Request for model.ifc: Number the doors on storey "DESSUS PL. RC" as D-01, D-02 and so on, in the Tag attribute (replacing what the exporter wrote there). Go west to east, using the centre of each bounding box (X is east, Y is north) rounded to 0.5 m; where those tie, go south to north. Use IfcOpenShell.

First a look at what the model holds.

```python
import ifcopenshell
import ifcopenshell.util.element
import ifcopenshell.util.placement

model = ifcopenshell.open("model.ifc")
print(model.schema)
storey = next(s for s in model.by_type("IfcBuildingStorey") if s.Name == "DESSUS PL. RC")
doors = [e for e in ifcopenshell.util.element.get_decomposition(storey) if e.is_a("IfcDoor")]
for e in sorted(doors, key=lambda e: e.id()):
    origin = ifcopenshell.util.placement.get_local_placement(e.ObjectPlacement)[:3, 3]
    print(e.id(), e.Tag, e.Name, origin.round(2) + 0.0, sep=" | ")
```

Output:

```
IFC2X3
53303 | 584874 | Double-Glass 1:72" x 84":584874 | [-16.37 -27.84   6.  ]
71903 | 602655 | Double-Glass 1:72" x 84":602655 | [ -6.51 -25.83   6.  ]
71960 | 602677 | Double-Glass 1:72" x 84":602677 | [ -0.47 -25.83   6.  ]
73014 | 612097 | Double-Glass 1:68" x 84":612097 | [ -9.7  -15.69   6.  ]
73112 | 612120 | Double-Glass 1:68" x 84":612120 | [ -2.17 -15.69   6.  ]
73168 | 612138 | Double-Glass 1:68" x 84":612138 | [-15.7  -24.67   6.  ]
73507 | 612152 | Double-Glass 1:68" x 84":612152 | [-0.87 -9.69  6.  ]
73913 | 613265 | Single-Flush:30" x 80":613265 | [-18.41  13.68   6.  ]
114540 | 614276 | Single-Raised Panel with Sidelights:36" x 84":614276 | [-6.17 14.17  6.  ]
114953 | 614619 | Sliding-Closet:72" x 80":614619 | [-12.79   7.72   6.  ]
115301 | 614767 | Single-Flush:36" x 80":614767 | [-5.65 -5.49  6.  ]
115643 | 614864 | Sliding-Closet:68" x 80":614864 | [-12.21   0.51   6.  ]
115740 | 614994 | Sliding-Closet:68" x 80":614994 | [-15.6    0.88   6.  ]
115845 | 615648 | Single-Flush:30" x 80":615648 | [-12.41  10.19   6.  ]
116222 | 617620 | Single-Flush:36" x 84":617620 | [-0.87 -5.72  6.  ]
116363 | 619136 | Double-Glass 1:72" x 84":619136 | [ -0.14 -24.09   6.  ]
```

```python
import ifcopenshell
import ifcopenshell.geom
import ifcopenshell.util.element
import ifcopenshell.util.shape

model = ifcopenshell.open("model.ifc")
settings = ifcopenshell.geom.settings()
settings.set("use-world-coords", True)


def centre(element):
    shape = ifcopenshell.geom.create_shape(settings, element)
    return ifcopenshell.util.shape.get_bbox_centroid(shape.geometry)


storey = next(s for s in model.by_type("IfcBuildingStorey") if s.Name == "DESSUS PL. RC")
doors = [e for e in ifcopenshell.util.element.get_decomposition(storey) if e.is_a("IfcDoor")]

# Insertion points can sit at a corner or the storey origin, so sort by the geometry (in metres).
centres = {e: centre(e) for e in doors}
doors.sort(key=lambda e: (round(centres[e][0] / 0.5), centres[e][1]))

for i, e in enumerate(doors, start=1):
    number = f"D-{i:02d}"
    e.Tag = number
    print(e.id(), number)

model.write("model_v2.ifc")
```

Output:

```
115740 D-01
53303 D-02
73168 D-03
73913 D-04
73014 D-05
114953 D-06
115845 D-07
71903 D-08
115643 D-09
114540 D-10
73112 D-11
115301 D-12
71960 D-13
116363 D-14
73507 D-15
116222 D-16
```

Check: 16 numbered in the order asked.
